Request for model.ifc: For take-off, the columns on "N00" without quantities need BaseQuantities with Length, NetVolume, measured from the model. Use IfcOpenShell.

First a look at what the model holds.

```python
import ifcopenshell
import ifcopenshell.util.element
import ifcopenshell.util.unit

model = ifcopenshell.open("model.ifc")
print(model.schema)
for unit_type in ("LENGTHUNIT", "AREAUNIT", "VOLUMEUNIT"):
    print(unit_type, ifcopenshell.util.unit.calculate_unit_scale(model, unit_type))
storey = next(s for s in model.by_type("IfcBuildingStorey") if s.Name == "N00")
columns = [e for e in ifcopenshell.util.element.get_decomposition(storey) if e.is_a("IfcColumn")]
for e in sorted(columns, key=lambda e: e.id()):
    print(e.id(), e.is_a(), e.Name, list(ifcopenshell.util.element.get_psets(e, qtos_only=True)), sep=" | ")
```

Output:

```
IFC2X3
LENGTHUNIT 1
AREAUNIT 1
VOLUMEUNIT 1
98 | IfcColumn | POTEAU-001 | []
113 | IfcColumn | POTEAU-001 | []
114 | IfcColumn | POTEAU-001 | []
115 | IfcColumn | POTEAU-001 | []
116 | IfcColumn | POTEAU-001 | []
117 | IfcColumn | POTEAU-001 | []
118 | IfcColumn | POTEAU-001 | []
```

```python
import ifcopenshell
import ifcopenshell.api.pset
import ifcopenshell.geom
import ifcopenshell.util.element
import ifcopenshell.util.shape
import ifcopenshell.util.unit

model = ifcopenshell.open("model.ifc")
unit_scale = ifcopenshell.util.unit.calculate_unit_scale(model)
volume_scale = ifcopenshell.util.unit.calculate_unit_scale(model, "VOLUMEUNIT")
settings = ifcopenshell.geom.settings()

storey = next(s for s in model.by_type("IfcBuildingStorey") if s.Name == "N00")
columns = [e for e in ifcopenshell.util.element.get_decomposition(storey) if e.is_a("IfcColumn")]

for e in sorted(columns, key=lambda e: e.id()):
    if ifcopenshell.util.element.get_psets(e, qtos_only=True, should_inherit=False):
        continue
    # Geometry comes back in metres, in the element's own axes.
    shape = ifcopenshell.geom.create_shape(settings, e)
    values = {
        "Length": ifcopenshell.util.shape.get_z(shape.geometry) / unit_scale,
        "NetVolume": ifcopenshell.util.shape.get_volume(shape.geometry) / volume_scale,
    }
    qto = ifcopenshell.api.pset.add_qto(model, product=e, name="BaseQuantities")
    ifcopenshell.api.pset.edit_qto(model, qto=qto, properties=values)
    print(e.id(), {k: round(v, 3) for k, v in values.items()})

model.write("model_updated.ifc")
```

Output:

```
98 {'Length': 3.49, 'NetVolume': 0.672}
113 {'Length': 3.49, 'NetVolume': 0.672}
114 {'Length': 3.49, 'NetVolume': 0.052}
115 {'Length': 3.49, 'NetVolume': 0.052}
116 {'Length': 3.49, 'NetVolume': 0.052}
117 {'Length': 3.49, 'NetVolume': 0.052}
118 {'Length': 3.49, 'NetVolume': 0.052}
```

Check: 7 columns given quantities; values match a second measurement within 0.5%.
